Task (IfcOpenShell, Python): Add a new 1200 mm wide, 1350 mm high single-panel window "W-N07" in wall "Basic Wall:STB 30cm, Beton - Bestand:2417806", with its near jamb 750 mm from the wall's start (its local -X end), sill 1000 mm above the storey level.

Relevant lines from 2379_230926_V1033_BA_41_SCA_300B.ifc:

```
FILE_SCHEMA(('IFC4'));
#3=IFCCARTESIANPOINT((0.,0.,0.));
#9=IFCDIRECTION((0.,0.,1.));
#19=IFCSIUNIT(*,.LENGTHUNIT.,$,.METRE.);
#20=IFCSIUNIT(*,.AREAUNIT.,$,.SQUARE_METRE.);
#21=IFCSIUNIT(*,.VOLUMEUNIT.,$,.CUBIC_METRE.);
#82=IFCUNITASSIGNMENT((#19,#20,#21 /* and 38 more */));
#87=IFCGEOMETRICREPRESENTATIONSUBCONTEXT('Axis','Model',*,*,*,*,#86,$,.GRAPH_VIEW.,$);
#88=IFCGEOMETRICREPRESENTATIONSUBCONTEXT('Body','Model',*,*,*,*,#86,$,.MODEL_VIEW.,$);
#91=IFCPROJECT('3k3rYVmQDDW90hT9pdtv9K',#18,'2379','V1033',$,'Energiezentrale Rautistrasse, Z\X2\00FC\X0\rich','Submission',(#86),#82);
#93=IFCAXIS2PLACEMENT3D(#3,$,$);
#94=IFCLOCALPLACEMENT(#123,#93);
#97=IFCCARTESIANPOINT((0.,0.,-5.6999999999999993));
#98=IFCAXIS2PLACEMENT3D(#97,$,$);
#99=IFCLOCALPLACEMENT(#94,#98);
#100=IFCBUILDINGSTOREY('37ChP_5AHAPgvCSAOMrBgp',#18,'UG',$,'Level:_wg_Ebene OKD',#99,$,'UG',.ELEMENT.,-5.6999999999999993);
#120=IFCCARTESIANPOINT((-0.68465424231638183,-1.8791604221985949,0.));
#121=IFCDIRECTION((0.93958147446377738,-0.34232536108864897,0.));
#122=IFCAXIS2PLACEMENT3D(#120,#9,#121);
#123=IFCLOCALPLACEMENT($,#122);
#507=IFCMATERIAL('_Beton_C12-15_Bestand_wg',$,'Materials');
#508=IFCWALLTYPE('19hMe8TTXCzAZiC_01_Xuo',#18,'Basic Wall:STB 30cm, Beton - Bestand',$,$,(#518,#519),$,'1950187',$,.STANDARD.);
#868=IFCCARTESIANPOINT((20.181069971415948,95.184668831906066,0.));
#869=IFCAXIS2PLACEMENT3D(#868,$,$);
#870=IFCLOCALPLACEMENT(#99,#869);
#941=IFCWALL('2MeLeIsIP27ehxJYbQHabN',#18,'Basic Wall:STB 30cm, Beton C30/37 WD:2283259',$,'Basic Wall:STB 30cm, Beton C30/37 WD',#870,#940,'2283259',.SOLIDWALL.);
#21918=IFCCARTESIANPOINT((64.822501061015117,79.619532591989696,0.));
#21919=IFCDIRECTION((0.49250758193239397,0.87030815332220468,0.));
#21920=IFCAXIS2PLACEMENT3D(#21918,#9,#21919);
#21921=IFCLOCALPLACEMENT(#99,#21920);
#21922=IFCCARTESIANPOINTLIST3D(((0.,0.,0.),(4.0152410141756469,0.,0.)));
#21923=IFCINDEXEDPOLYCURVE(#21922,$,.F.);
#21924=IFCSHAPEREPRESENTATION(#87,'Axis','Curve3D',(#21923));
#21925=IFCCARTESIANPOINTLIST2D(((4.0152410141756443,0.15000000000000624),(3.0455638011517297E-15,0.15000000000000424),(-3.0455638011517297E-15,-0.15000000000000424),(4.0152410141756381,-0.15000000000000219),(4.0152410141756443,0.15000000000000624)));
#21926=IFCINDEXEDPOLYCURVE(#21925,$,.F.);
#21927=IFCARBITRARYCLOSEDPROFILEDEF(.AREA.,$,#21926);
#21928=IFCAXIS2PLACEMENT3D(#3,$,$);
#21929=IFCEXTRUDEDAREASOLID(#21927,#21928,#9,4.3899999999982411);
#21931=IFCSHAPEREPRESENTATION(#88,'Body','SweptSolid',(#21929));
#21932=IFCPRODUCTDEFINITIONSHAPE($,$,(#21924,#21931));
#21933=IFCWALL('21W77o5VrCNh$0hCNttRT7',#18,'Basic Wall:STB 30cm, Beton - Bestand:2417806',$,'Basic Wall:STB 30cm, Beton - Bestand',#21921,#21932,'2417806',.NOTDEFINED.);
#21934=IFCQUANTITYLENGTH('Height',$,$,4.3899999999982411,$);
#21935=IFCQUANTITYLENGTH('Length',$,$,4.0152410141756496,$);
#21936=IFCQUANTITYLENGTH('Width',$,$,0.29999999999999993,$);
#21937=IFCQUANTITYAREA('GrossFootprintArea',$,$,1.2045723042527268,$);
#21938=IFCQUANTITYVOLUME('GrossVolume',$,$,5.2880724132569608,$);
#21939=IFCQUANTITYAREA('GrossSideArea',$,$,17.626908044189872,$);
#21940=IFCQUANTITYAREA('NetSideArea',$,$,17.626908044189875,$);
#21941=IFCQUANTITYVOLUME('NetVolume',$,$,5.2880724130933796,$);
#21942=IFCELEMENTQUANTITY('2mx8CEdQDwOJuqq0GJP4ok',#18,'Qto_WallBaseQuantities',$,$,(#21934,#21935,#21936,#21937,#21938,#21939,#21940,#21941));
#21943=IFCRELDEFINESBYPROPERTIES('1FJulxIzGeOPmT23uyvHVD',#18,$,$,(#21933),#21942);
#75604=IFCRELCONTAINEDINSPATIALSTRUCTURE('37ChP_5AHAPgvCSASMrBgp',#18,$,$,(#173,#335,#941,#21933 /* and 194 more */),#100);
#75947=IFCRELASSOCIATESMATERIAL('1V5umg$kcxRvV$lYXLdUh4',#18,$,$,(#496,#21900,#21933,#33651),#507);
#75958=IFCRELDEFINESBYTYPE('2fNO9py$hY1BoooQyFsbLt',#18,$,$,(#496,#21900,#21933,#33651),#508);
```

```python
import numpy as np
import ifcopenshell
import ifcopenshell.api.feature
import ifcopenshell.api.geometry
import ifcopenshell.api.pset
import ifcopenshell.api.root
import ifcopenshell.api.spatial
import ifcopenshell.geom
import ifcopenshell.util.element
import ifcopenshell.util.placement
import ifcopenshell.util.representation
import ifcopenshell.util.shape
import ifcopenshell.util.unit

model = ifcopenshell.open("2379_230926_V1033_BA_41_SCA_300B.ifc")
unit_scale = ifcopenshell.util.unit.calculate_unit_scale(model)
area_scale = ifcopenshell.util.unit.calculate_unit_scale(model, "AREAUNIT")
volume_scale = ifcopenshell.util.unit.calculate_unit_scale(model, "VOLUMEUNIT")
settings = ifcopenshell.geom.settings()


def volume(element):
    """Net volume in cubic metres, openings subtracted."""
    shape = ifcopenshell.geom.create_shape(settings, element)
    return ifcopenshell.util.shape.get_volume(shape.geometry)


wall = model.by_id(21933)
storey = ifcopenshell.util.element.get_container(wall, ifc_class="IfcBuildingStorey")
context = ifcopenshell.util.representation.get_context(model, "Model", "Body", "MODEL_VIEW")
before = volume(wall)

width, height, from_end, sill = 1.2, 1.35, 0.75, 1  # metres

# The wall runs along its own X axis, and the end named is its -X end.
wall_shape = ifcopenshell.geom.create_shape(settings, wall)
x, y, z = ifcopenshell.util.shape.get_vertices(wall_shape.geometry).T
start = x.min() + from_end
face, thickness = float(y.min()), float(y.max() - y.min())
wall_matrix = ifcopenshell.util.placement.get_local_placement(wall.ObjectPlacement)
level = ifcopenshell.util.placement.get_local_placement(storey.ObjectPlacement)[2, 3]


def in_wall(x, y):
    """Placement at x, y metres in the wall's axes, at sill height."""
    matrix = wall_matrix.copy()
    matrix[:, 3] = wall_matrix @ np.array([x / unit_scale, y / unit_scale, 0.0, 1.0])
    matrix[2, 3] = level + sill / unit_scale
    return matrix


# Opening: a box that overshoots both wall faces by 50 mm.
opening = ifcopenshell.api.root.create_entity(model, ifc_class="IfcOpeningElement", predefined_type="OPENING")
box = ifcopenshell.api.geometry.add_wall_representation(
    model, context=context, length=width, height=height, thickness=thickness + 0.1
)
ifcopenshell.api.geometry.assign_representation(model, product=opening, representation=box)
ifcopenshell.api.geometry.edit_object_placement(model, product=opening, matrix=in_wall(start, face - 0.05), is_si=False)
ifcopenshell.api.feature.add_feature(model, feature=opening, element=wall)

window = ifcopenshell.api.root.create_entity(model, ifc_class="IfcWindow", name="W-N07", predefined_type="WINDOW")
window.OverallWidth, window.OverallHeight = width / unit_scale, height / unit_scale
window.PartitioningType = "SINGLE_PANEL"
body = ifcopenshell.api.geometry.add_window_representation(
    model,
    context=context,
    overall_width=window.OverallWidth,
    overall_height=window.OverallHeight,
    partition_type="SINGLE_PANEL",
)
ifcopenshell.api.geometry.assign_representation(model, product=window, representation=body)
ifcopenshell.api.spatial.assign_container(model, products=[window], relating_structure=storey)
ifcopenshell.api.feature.add_filling(model, opening=opening, element=window)

# Centre the window in the wall's thickness.
ifcopenshell.api.geometry.edit_object_placement(model, product=window, matrix=in_wall(start, face), is_si=False)
window_shape = ifcopenshell.geom.create_shape(settings, window)
depth = ifcopenshell.util.shape.get_vertices(window_shape.geometry)[:, 1]
offset = face + thickness / 2 - (depth.min() + depth.max()) / 2
ifcopenshell.api.geometry.edit_object_placement(model, product=window, matrix=in_wall(start, offset), is_si=False)

after = volume(wall)

# Update the wall's stored quantities.
qto = model.by_id(ifcopenshell.util.element.get_pset(wall, "Qto_WallBaseQuantities", should_inherit=False)["id"])
ifcopenshell.api.pset.edit_qto(model, qto=qto, properties={
    "NetSideArea": after / thickness / area_scale,
    "NetVolume": after / volume_scale,
})

print(f"wall volume {before:.3f} -> {after:.3f} m3")

model.write("2379_230926_V1033_BA_41_SCA_300B_rev.ifc")
```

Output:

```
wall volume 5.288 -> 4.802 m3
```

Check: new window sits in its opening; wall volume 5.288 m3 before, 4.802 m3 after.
